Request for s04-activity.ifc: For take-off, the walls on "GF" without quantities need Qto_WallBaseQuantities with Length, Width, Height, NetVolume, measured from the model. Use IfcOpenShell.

First a look at what the model holds.

```python
import ifcopenshell
import ifcopenshell.util.element
import ifcopenshell.util.unit

model = ifcopenshell.open("s04-activity.ifc")
print(model.schema)
for unit_type in ("LENGTHUNIT", "AREAUNIT", "VOLUMEUNIT"):
    print(unit_type, ifcopenshell.util.unit.calculate_unit_scale(model, unit_type))
storey = next(s for s in model.by_type("IfcBuildingStorey") if s.Name == "GF")
walls = [e for e in ifcopenshell.util.element.get_decomposition(storey) if e.is_a("IfcWall")]
for e in sorted(walls, key=lambda e: e.id()):
    print(e.id(), e.is_a(), e.Name, list(ifcopenshell.util.element.get_psets(e, qtos_only=True)), sep=" | ")
```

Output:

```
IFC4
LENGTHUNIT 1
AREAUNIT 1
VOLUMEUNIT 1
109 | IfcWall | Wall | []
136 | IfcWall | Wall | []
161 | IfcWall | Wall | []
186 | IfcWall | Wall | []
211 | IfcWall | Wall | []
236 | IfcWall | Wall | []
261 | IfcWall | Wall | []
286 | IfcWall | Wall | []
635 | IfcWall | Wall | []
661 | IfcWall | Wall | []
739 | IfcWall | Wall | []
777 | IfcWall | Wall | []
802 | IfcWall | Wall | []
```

```python
import ifcopenshell
import ifcopenshell.api.pset
import ifcopenshell.geom
import ifcopenshell.util.element
import ifcopenshell.util.shape
import ifcopenshell.util.unit

model = ifcopenshell.open("s04-activity.ifc")
unit_scale = ifcopenshell.util.unit.calculate_unit_scale(model)
volume_scale = ifcopenshell.util.unit.calculate_unit_scale(model, "VOLUMEUNIT")
settings = ifcopenshell.geom.settings()

storey = next(s for s in model.by_type("IfcBuildingStorey") if s.Name == "GF")
walls = [e for e in ifcopenshell.util.element.get_decomposition(storey) if e.is_a("IfcWall")]

for e in sorted(walls, key=lambda e: e.id()):
    if ifcopenshell.util.element.get_psets(e, qtos_only=True, should_inherit=False):
        continue
    # Geometry comes back in metres, in the element's own axes.
    shape = ifcopenshell.geom.create_shape(settings, e)
    values = {
        "Length": ifcopenshell.util.shape.get_x(shape.geometry) / unit_scale,
        "Width": ifcopenshell.util.shape.get_y(shape.geometry) / unit_scale,
        "Height": ifcopenshell.util.shape.get_z(shape.geometry) / unit_scale,
        "NetVolume": ifcopenshell.util.shape.get_volume(shape.geometry) / volume_scale,
    }
    qto = ifcopenshell.api.pset.add_qto(model, product=e, name="Qto_WallBaseQuantities")
    ifcopenshell.api.pset.edit_qto(model, qto=qto, properties=values)
    print(e.id(), {k: round(v, 3) for k, v in values.items()})

model.write("s04-activity_updated.ifc")
```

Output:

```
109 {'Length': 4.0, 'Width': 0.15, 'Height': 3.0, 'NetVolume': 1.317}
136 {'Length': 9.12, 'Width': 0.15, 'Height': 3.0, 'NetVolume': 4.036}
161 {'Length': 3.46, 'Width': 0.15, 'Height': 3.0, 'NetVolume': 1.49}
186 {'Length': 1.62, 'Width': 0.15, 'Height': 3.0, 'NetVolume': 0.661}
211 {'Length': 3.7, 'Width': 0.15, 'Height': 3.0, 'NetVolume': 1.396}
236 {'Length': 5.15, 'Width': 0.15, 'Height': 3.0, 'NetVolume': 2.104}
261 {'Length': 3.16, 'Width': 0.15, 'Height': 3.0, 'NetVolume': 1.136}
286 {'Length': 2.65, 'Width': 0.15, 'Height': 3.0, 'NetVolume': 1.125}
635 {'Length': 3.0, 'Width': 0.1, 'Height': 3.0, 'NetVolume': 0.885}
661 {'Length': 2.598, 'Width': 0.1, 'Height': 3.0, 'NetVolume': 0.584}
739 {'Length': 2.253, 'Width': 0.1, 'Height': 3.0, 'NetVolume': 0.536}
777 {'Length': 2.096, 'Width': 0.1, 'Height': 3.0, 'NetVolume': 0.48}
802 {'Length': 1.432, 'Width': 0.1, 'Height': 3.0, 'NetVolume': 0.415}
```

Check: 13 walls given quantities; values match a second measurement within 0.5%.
